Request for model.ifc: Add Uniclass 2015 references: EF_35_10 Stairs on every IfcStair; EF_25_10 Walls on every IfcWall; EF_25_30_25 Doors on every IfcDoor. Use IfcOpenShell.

First a look at what the model holds.

```python
import ifcopenshell

model = ifcopenshell.open("model.ifc")
print(model.schema)
print("classifications:", [c.Name for c in model.by_type("IfcClassification")])
for ifc_class in ("IfcDoor", "IfcRoof", "IfcStair", "IfcWall", "IfcWindow"):
    print(ifc_class, len(model.by_type(ifc_class)))
```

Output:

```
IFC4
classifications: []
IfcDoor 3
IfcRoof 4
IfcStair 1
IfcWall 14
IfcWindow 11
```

```python
import ifcopenshell
import ifcopenshell.api.classification

model = ifcopenshell.open("model.ifc")

system = ifcopenshell.api.classification.add_classification(model, classification="Uniclass 2015")

codes = {
    "IfcStair": ("EF_35_10", "Stairs"),
    "IfcWall": ("EF_25_10", "Walls"),
    "IfcDoor": ("EF_25_30_25", "Doors"),
}
for ifc_class, (code, name) in codes.items():
    products = model.by_type(ifc_class)
    ifcopenshell.api.classification.add_reference(
        model, products=products, classification=system, identification=code, name=name
    )
    print(code, len(products))

model.write("model_v2.ifc")
```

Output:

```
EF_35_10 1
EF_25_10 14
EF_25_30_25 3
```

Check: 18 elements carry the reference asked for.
